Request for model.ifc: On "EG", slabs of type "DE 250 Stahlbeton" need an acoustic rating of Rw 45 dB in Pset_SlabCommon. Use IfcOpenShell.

First a look at what the model holds.

```python
import ifcopenshell
import ifcopenshell.util.element

model = ifcopenshell.open("model.ifc")
print(model.schema)
storey = next(s for s in model.by_type("IfcBuildingStorey") if s.Name == "EG")
slabs = [e for e in ifcopenshell.util.element.get_decomposition(storey) if e.is_a("IfcSlab")]
seen = {}
for e in slabs:
    element_type = ifcopenshell.util.element.get_type(e)
    key = (element_type.Name if element_type != e and element_type else None, ifcopenshell.util.element.get_pset(e, "Pset_SlabCommon", "AcousticRating"))
    seen[key] = seen.get(key, 0) + 1
for (name, value), count in sorted(seen.items(), key=str):
    print(count, "x", name, "|", value)
```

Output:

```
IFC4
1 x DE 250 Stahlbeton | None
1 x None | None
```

```python
import ifcopenshell
import ifcopenshell.api.pset
import ifcopenshell.util.element

model = ifcopenshell.open("model.ifc")

storey = next(s for s in model.by_type("IfcBuildingStorey") if s.Name == "EG")
slabs = [e for e in ifcopenshell.util.element.get_decomposition(storey) if e.is_a("IfcSlab")]

count = 0
for e in slabs:
    element_type = ifcopenshell.util.element.get_type(e)
    if element_type in (None, e) or element_type.Name != "DE 250 Stahlbeton":
        continue
    # add_pset returns the element's existing set when there is one.
    pset = ifcopenshell.api.pset.add_pset(model, product=e, name="Pset_SlabCommon")
    ifcopenshell.api.pset.edit_pset(model, pset=pset, properties={"AcousticRating": "Rw 45 dB"})
    count += 1

print(count, "slabs updated")

model.write("model_rev.ifc")
```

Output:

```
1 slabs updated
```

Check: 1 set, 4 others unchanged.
